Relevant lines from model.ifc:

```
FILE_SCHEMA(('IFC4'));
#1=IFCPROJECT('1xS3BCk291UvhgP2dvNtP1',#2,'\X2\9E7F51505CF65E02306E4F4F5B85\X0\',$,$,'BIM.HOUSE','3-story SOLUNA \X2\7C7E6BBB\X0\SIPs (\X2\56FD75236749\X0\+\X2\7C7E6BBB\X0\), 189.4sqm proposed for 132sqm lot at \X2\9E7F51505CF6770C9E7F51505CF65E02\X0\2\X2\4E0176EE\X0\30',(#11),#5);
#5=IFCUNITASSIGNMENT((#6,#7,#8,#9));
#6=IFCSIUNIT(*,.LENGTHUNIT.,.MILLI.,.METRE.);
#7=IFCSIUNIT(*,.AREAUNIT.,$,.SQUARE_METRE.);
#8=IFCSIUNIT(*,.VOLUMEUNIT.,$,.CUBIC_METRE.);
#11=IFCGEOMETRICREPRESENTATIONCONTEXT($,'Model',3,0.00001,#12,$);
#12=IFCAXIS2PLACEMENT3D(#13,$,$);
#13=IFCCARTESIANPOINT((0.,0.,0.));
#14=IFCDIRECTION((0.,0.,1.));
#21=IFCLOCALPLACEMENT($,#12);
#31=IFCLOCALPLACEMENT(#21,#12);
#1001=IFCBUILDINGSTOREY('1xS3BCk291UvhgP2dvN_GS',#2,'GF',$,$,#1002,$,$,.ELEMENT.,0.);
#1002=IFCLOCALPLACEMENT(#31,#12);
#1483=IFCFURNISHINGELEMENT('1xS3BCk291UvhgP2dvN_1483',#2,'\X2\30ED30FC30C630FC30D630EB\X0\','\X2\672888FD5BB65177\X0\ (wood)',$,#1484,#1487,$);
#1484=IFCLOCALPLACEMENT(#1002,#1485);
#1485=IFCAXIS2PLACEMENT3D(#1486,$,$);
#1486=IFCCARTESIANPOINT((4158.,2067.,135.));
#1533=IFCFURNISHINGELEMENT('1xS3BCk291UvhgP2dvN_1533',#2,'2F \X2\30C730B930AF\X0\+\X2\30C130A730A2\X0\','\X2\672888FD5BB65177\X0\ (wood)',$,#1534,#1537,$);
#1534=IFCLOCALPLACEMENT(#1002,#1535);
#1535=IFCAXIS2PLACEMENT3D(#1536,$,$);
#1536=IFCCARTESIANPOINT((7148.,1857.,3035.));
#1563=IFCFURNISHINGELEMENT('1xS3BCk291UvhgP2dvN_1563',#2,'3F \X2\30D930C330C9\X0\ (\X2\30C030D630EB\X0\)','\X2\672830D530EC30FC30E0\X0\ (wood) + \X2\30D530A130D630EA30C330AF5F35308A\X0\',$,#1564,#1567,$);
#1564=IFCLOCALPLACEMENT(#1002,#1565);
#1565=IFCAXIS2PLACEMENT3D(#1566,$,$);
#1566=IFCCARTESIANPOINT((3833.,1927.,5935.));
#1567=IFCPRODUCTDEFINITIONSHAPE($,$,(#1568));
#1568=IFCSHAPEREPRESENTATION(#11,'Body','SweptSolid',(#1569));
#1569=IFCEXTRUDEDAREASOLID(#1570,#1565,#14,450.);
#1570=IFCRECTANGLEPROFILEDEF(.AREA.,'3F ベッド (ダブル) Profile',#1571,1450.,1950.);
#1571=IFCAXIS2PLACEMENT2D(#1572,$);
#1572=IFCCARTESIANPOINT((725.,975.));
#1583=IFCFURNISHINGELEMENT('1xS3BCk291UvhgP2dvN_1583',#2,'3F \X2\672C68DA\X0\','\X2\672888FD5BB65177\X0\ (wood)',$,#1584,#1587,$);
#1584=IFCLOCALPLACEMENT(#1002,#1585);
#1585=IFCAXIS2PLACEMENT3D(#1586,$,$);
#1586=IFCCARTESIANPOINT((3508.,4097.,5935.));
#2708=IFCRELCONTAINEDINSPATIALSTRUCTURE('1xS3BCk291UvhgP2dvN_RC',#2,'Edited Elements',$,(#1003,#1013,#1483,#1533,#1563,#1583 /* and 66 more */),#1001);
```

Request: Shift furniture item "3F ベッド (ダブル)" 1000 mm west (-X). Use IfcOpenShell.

```python
import ifcopenshell
import ifcopenshell.api.geometry
import ifcopenshell.util.placement
import ifcopenshell.util.unit

model = ifcopenshell.open("model.ifc")
unit_scale = ifcopenshell.util.unit.calculate_unit_scale(model)

item = model.by_guid("1xS3BCk291UvhgP2dvN_1563")
matrix = ifcopenshell.util.placement.get_local_placement(item.ObjectPlacement)
matrix[0, 3] -= 1 / unit_scale
ifcopenshell.api.geometry.edit_object_placement(model, product=item, matrix=matrix, is_si=False)

print(ifcopenshell.util.placement.get_local_placement(item.ObjectPlacement).round(3) + 0.0)

model.write("model_edited.ifc")
```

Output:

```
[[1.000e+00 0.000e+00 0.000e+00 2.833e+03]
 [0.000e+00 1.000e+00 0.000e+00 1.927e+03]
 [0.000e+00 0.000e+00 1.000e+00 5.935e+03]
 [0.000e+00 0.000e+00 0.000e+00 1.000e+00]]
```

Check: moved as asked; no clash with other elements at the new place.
